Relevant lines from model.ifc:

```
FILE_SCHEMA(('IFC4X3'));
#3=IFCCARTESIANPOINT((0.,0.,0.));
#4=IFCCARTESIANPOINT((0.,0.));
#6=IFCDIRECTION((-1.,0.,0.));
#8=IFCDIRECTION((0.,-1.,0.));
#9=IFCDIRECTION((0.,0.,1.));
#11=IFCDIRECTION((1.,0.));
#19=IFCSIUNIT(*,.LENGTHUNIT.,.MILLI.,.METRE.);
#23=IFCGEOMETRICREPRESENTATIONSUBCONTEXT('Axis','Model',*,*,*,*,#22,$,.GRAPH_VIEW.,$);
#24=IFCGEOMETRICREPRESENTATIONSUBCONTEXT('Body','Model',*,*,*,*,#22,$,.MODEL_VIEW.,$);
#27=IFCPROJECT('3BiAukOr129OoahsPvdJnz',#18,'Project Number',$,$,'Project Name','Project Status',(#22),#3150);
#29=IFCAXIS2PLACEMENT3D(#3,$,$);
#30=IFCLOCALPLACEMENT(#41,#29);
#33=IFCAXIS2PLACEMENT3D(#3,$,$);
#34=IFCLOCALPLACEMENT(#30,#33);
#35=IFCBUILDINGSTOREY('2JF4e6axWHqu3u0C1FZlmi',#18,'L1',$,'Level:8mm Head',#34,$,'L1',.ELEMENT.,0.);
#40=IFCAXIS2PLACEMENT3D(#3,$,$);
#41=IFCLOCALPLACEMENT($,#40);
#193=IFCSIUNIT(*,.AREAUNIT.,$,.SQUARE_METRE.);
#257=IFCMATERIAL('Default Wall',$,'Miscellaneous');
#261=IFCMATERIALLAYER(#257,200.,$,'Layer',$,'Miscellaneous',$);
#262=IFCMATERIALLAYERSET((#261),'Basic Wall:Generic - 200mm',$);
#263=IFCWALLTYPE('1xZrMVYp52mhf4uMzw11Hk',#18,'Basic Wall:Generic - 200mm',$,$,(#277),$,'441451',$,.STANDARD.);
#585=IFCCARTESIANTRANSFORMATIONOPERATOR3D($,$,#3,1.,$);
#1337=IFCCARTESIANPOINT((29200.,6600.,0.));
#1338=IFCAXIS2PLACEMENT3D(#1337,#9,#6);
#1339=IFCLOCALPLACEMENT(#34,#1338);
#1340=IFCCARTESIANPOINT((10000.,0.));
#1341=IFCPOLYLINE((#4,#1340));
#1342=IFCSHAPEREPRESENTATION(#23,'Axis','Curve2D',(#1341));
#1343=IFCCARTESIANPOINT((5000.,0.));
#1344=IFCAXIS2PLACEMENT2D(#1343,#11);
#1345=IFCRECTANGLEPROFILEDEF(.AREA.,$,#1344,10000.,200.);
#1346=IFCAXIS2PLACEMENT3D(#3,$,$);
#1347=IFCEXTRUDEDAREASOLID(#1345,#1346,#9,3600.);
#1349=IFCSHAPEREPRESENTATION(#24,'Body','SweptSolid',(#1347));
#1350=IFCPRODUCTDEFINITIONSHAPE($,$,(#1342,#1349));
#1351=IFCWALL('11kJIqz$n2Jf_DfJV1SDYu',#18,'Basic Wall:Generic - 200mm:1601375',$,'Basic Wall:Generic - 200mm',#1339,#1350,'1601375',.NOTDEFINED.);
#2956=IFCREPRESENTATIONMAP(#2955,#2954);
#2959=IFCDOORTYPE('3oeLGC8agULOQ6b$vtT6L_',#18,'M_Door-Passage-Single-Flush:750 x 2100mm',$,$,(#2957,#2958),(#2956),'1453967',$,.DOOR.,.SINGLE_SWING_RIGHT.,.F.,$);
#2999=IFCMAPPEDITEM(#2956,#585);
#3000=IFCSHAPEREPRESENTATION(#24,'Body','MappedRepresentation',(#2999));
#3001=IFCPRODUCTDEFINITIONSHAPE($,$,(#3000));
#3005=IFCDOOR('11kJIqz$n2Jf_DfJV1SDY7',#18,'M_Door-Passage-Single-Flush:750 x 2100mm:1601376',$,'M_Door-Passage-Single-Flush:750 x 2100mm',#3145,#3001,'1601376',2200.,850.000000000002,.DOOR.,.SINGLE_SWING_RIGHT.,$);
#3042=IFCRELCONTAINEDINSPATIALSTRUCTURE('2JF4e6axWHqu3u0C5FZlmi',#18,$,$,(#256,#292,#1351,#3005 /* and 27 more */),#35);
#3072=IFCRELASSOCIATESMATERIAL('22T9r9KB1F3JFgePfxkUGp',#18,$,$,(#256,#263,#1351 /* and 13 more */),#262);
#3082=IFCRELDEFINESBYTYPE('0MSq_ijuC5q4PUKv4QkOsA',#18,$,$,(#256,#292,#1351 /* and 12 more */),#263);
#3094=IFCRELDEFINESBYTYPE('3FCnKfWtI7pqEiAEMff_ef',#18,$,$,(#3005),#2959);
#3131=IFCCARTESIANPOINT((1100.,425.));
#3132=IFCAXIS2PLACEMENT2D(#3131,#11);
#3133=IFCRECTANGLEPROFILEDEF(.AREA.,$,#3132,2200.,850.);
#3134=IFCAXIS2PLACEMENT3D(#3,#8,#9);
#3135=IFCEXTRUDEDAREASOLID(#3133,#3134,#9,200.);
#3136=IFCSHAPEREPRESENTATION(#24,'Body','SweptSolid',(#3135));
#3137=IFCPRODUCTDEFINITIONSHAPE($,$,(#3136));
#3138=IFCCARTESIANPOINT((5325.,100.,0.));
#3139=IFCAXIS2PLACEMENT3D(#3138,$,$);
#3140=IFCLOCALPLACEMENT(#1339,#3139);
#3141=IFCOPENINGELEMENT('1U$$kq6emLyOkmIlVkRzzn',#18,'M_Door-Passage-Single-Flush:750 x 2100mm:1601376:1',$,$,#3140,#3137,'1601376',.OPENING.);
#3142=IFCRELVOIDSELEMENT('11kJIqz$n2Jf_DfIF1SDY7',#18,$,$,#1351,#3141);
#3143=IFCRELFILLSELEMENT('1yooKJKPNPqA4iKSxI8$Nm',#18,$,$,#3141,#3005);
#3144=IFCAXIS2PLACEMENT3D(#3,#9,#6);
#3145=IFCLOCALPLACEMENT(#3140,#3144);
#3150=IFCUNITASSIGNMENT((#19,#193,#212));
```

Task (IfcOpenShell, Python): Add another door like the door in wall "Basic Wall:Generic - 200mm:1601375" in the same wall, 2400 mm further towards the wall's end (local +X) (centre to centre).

```python
import ifcopenshell
import ifcopenshell.api.feature
import ifcopenshell.api.geometry
import ifcopenshell.api.root
import ifcopenshell.geom
import ifcopenshell.util.element
import ifcopenshell.util.placement
import ifcopenshell.util.shape
import ifcopenshell.util.unit

model = ifcopenshell.open("model.ifc")
unit_scale = ifcopenshell.util.unit.calculate_unit_scale(model)
settings = ifcopenshell.geom.settings()


def volume(element):
    """Net volume in cubic metres, openings subtracted."""
    shape = ifcopenshell.geom.create_shape(settings, element)
    return ifcopenshell.util.shape.get_volume(shape.geometry)


def reuse_history(source, copy):
    """copy_class also copies each property set's owner history, people and application; keep the originals."""
    for rel in copy.IsDefinedBy:
        if rel.is_a("IfcRelDefinesByProperties") and (history := rel.RelatingPropertyDefinition.OwnerHistory):
            rel.RelatingPropertyDefinition.OwnerHistory = source.OwnerHistory
            ifcopenshell.util.element.remove_deep2(model, history)


door = model.by_guid("11kJIqz$n2Jf_DfJV1SDY7")
opening = door.FillsVoids[0].RelatingOpeningElement
wall = opening.VoidsElements[0].RelatingBuildingElement
before = volume(wall)
shift = ifcopenshell.util.placement.get_local_placement(wall.ObjectPlacement)[:3, 0] * 2.4 / unit_scale

# copy_class copies the void relationship, type, container and properties, but no geometry.
new_opening = ifcopenshell.api.root.copy_class(model, product=opening)
new_opening.Representation = ifcopenshell.util.element.copy_deep(
    model, opening.Representation, exclude=["IfcGeometricRepresentationContext", "IfcRepresentationMap"]
)
new_opening.Name = "M_Door-Passage-Single-Flush:750 x 2100mm"
new_opening.Tag = None
new_door = ifcopenshell.api.root.copy_class(model, product=door)
new_door.Representation = ifcopenshell.util.element.copy_deep(
    model, door.Representation, exclude=["IfcGeometricRepresentationContext", "IfcRepresentationMap"]
)
new_door.Name = "M_Door-Passage-Single-Flush:750 x 2100mm"
new_door.Tag = None
reuse_history(door, new_door)
ifcopenshell.api.feature.add_filling(model, opening=new_opening, element=new_door)

for old, new in ((opening, new_opening), (door, new_door)):
    matrix = ifcopenshell.util.placement.get_local_placement(old.ObjectPlacement)
    matrix[:3, 3] += shift
    ifcopenshell.api.geometry.edit_object_placement(model, product=new, matrix=matrix, is_si=False)

after = volume(wall)

print(f"wall volume {before:.3f} -> {after:.3f} m3")

model.write("model_edited.ifc")
```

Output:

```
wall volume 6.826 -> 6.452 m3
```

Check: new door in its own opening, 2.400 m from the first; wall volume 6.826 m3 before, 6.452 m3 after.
